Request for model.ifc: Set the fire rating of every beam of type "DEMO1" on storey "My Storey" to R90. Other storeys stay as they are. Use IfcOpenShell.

First a look at what the model holds.

```python
import ifcopenshell
import ifcopenshell.util.element

model = ifcopenshell.open("model.ifc")
print(model.schema)
storey = next(s for s in model.by_type("IfcBuildingStorey") if s.Name == "My Storey")
beams = [e for e in ifcopenshell.util.element.get_decomposition(storey) if e.is_a("IfcBeam")]
seen = {}
for e in beams:
    element_type = ifcopenshell.util.element.get_type(e)
    key = (element_type.Name if element_type != e and element_type else None, ifcopenshell.util.element.get_pset(e, "Pset_BeamCommon", "FireRating"))
    seen[key] = seen.get(key, 0) + 1
for (name, value), count in sorted(seen.items(), key=str):
    print(count, "x", name, "|", value)
```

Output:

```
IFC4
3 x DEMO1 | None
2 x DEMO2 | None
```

```python
import ifcopenshell
import ifcopenshell.api.pset
import ifcopenshell.util.element

model = ifcopenshell.open("model.ifc")

storey = next(s for s in model.by_type("IfcBuildingStorey") if s.Name == "My Storey")
beams = [e for e in ifcopenshell.util.element.get_decomposition(storey) if e.is_a("IfcBeam")]

count = 0
for e in beams:
    element_type = ifcopenshell.util.element.get_type(e)
    if element_type in (None, e) or element_type.Name != "DEMO1":
        continue
    # add_pset returns the element's existing set when there is one.
    pset = ifcopenshell.api.pset.add_pset(model, product=e, name="Pset_BeamCommon")
    ifcopenshell.api.pset.edit_pset(model, pset=pset, properties={"FireRating": "R90"})
    count += 1

print(count, "beams updated")

model.write("model_edited.ifc")
```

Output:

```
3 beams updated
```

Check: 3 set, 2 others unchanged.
